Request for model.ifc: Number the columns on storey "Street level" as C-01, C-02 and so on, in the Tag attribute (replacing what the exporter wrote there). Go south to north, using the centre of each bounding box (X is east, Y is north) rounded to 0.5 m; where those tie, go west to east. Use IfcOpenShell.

First a look at what the model holds.

```python
import ifcopenshell
import ifcopenshell.util.element
import ifcopenshell.util.placement

model = ifcopenshell.open("model.ifc")
print(model.schema)
storey = next(s for s in model.by_type("IfcBuildingStorey") if s.Name == "Street level")
columns = [e for e in ifcopenshell.util.element.get_decomposition(storey) if e.is_a("IfcColumn")]
for e in sorted(columns, key=lambda e: e.id()):
    origin = ifcopenshell.util.placement.get_local_placement(e.ObjectPlacement)[:3, 3]
    print(e.id(), e.Tag, e.Name, origin.round(2) + 0.0, sep=" | ")
```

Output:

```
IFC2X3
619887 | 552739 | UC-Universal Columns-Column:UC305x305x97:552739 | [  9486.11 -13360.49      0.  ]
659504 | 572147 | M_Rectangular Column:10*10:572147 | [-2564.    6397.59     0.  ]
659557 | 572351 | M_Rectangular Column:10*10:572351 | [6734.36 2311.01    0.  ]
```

```python
import ifcopenshell
import ifcopenshell.geom
import ifcopenshell.util.element
import ifcopenshell.util.shape

model = ifcopenshell.open("model.ifc")
settings = ifcopenshell.geom.settings()
settings.set("use-world-coords", True)


def centre(element):
    shape = ifcopenshell.geom.create_shape(settings, element)
    return ifcopenshell.util.shape.get_bbox_centroid(shape.geometry)


storey = next(s for s in model.by_type("IfcBuildingStorey") if s.Name == "Street level")
columns = [e for e in ifcopenshell.util.element.get_decomposition(storey) if e.is_a("IfcColumn")]

# Insertion points can sit at a corner or the storey origin, so sort by the geometry (in metres).
centres = {e: centre(e) for e in columns}
columns.sort(key=lambda e: (round(centres[e][1] / 0.5), centres[e][0]))

for i, e in enumerate(columns, start=1):
    number = f"C-{i:02d}"
    e.Tag = number
    print(e.id(), number)

model.write("model_updated.ifc")
```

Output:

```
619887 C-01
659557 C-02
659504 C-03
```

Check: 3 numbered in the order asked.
